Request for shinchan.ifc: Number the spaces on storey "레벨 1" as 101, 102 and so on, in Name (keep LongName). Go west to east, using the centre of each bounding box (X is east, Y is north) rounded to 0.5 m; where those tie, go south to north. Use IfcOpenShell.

First a look at what the model holds.

```python
import ifcopenshell
import ifcopenshell.util.element
import ifcopenshell.util.placement

model = ifcopenshell.open("shinchan.ifc")
print(model.schema)
storey = next(s for s in model.by_type("IfcBuildingStorey") if s.Name == "레벨 1")
spaces = [e for e in ifcopenshell.util.element.get_decomposition(storey) if e.is_a("IfcSpace")]
for e in sorted(spaces, key=lambda e: e.id()):
    origin = ifcopenshell.util.placement.get_local_placement(e.ObjectPlacement)[:3, 3]
    print(e.id(), e.Name, e.LongName, origin.round(2) + 0.0, sep=" | ")
```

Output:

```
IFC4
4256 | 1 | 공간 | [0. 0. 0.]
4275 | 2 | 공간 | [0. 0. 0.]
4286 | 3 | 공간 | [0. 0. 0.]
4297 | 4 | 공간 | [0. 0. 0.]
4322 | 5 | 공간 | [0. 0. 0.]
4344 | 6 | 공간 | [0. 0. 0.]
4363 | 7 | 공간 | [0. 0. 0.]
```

```python
import ifcopenshell
import ifcopenshell.geom
import ifcopenshell.util.element
import ifcopenshell.util.shape

model = ifcopenshell.open("shinchan.ifc")
settings = ifcopenshell.geom.settings()
settings.set("use-world-coords", True)


def centre(element):
    shape = ifcopenshell.geom.create_shape(settings, element)
    return ifcopenshell.util.shape.get_bbox_centroid(shape.geometry)


storey = next(s for s in model.by_type("IfcBuildingStorey") if s.Name == "레벨 1")
spaces = [e for e in ifcopenshell.util.element.get_decomposition(storey) if e.is_a("IfcSpace")]

# Insertion points can sit at a corner or the storey origin, so sort by the geometry (in metres).
centres = {e: centre(e) for e in spaces}
spaces.sort(key=lambda e: (round(centres[e][0] / 0.5), centres[e][1]))

for i, e in enumerate(spaces, start=1):
    number = f"1{i:02d}"
    e.Name = number
    print(e.id(), number)

model.write("shinchan_edited.ifc")
```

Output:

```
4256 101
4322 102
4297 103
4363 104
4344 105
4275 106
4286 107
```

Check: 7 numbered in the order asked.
